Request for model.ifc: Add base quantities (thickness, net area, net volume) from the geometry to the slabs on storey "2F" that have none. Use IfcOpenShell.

First a look at what the model holds.

```python
import ifcopenshell
import ifcopenshell.util.element
import ifcopenshell.util.unit

model = ifcopenshell.open("model.ifc")
print(model.schema)
for unit_type in ("LENGTHUNIT", "AREAUNIT", "VOLUMEUNIT"):
    print(unit_type, ifcopenshell.util.unit.calculate_unit_scale(model, unit_type))
storey = next(s for s in model.by_type("IfcBuildingStorey") if s.Name == "2F")
slabs = [e for e in ifcopenshell.util.element.get_decomposition(storey) if e.is_a("IfcSlab")]
for e in sorted(slabs, key=lambda e: e.id()):
    print(e.id(), e.is_a(), e.Name, list(ifcopenshell.util.element.get_psets(e, qtos_only=True)), sep=" | ")
```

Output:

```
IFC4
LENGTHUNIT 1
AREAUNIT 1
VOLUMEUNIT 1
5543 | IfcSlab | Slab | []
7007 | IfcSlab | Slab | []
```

```python
import ifcopenshell
import ifcopenshell.api.pset
import ifcopenshell.geom
import ifcopenshell.util.element
import ifcopenshell.util.shape
import ifcopenshell.util.unit

model = ifcopenshell.open("model.ifc")
unit_scale = ifcopenshell.util.unit.calculate_unit_scale(model)
area_scale = ifcopenshell.util.unit.calculate_unit_scale(model, "AREAUNIT")
volume_scale = ifcopenshell.util.unit.calculate_unit_scale(model, "VOLUMEUNIT")
settings = ifcopenshell.geom.settings()

storey = next(s for s in model.by_type("IfcBuildingStorey") if s.Name == "2F")
slabs = [e for e in ifcopenshell.util.element.get_decomposition(storey) if e.is_a("IfcSlab")]

for e in sorted(slabs, key=lambda e: e.id()):
    if ifcopenshell.util.element.get_psets(e, qtos_only=True, should_inherit=False):
        continue
    # Geometry comes back in metres, in the element's own axes.
    shape = ifcopenshell.geom.create_shape(settings, e)
    values = {
        "Width": ifcopenshell.util.shape.get_z(shape.geometry) / unit_scale,
        "NetArea": ifcopenshell.util.shape.get_footprint_area(shape.geometry) / area_scale,
        "NetVolume": ifcopenshell.util.shape.get_volume(shape.geometry) / volume_scale,
    }
    qto = ifcopenshell.api.pset.add_qto(model, product=e, name="Qto_SlabBaseQuantities")
    ifcopenshell.api.pset.edit_qto(model, qto=qto, properties=values)
    print(e.id(), {k: round(v, 3) for k, v in values.items()})

model.write("model_rev.ifc")
```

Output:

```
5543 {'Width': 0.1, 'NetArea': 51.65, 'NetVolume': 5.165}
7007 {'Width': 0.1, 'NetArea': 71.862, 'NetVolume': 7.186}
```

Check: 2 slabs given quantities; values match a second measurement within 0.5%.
